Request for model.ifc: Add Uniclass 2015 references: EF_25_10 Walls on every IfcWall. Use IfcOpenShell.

First a look at what the model holds.

```python
import ifcopenshell

model = ifcopenshell.open("model.ifc")
print(model.schema)
print("classifications:", [c.Name for c in model.by_type("IfcClassification")])
for ifc_class in ("IfcDoor", "IfcRoof", "IfcStair", "IfcWall", "IfcWindow"):
    print(ifc_class, len(model.by_type(ifc_class)))
```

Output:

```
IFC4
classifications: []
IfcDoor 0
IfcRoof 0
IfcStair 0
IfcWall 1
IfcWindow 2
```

```python
import ifcopenshell
import ifcopenshell.api.classification

model = ifcopenshell.open("model.ifc")

system = ifcopenshell.api.classification.add_classification(model, classification="Uniclass 2015")

codes = {
    "IfcWall": ("EF_25_10", "Walls"),
}
for ifc_class, (code, name) in codes.items():
    products = model.by_type(ifc_class)
    ifcopenshell.api.classification.add_reference(
        model, products=products, classification=system, identification=code, name=name
    )
    print(code, len(products))

model.write("model_updated.ifc")
```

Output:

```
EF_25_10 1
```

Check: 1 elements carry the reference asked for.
